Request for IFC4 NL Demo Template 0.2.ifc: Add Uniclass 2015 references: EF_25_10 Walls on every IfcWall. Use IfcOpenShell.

First a look at what the model holds.

```python
import ifcopenshell

model = ifcopenshell.open("IFC4 NL Demo Template 0.2.ifc")
print(model.schema)
print("classifications:", [c.Name for c in model.by_type("IfcClassification")])
for ifc_class in ("IfcDoor", "IfcRoof", "IfcStair", "IfcWall", "IfcWindow"):
    print(ifc_class, len(model.by_type(ifc_class)))
```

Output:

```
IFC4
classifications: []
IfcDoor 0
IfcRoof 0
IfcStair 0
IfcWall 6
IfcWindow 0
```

```python
import ifcopenshell
import ifcopenshell.api.classification

model = ifcopenshell.open("IFC4 NL Demo Template 0.2.ifc")

system = ifcopenshell.api.classification.add_classification(model, classification="Uniclass 2015")

codes = {
    "IfcWall": ("EF_25_10", "Walls"),
}
for ifc_class, (code, name) in codes.items():
    products = model.by_type(ifc_class)
    ifcopenshell.api.classification.add_reference(
        model, products=products, classification=system, identification=code, name=name
    )
    print(code, len(products))

model.write("IFC4 NL Demo Template 0.2_rev.ifc")
```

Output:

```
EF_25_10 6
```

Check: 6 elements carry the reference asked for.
